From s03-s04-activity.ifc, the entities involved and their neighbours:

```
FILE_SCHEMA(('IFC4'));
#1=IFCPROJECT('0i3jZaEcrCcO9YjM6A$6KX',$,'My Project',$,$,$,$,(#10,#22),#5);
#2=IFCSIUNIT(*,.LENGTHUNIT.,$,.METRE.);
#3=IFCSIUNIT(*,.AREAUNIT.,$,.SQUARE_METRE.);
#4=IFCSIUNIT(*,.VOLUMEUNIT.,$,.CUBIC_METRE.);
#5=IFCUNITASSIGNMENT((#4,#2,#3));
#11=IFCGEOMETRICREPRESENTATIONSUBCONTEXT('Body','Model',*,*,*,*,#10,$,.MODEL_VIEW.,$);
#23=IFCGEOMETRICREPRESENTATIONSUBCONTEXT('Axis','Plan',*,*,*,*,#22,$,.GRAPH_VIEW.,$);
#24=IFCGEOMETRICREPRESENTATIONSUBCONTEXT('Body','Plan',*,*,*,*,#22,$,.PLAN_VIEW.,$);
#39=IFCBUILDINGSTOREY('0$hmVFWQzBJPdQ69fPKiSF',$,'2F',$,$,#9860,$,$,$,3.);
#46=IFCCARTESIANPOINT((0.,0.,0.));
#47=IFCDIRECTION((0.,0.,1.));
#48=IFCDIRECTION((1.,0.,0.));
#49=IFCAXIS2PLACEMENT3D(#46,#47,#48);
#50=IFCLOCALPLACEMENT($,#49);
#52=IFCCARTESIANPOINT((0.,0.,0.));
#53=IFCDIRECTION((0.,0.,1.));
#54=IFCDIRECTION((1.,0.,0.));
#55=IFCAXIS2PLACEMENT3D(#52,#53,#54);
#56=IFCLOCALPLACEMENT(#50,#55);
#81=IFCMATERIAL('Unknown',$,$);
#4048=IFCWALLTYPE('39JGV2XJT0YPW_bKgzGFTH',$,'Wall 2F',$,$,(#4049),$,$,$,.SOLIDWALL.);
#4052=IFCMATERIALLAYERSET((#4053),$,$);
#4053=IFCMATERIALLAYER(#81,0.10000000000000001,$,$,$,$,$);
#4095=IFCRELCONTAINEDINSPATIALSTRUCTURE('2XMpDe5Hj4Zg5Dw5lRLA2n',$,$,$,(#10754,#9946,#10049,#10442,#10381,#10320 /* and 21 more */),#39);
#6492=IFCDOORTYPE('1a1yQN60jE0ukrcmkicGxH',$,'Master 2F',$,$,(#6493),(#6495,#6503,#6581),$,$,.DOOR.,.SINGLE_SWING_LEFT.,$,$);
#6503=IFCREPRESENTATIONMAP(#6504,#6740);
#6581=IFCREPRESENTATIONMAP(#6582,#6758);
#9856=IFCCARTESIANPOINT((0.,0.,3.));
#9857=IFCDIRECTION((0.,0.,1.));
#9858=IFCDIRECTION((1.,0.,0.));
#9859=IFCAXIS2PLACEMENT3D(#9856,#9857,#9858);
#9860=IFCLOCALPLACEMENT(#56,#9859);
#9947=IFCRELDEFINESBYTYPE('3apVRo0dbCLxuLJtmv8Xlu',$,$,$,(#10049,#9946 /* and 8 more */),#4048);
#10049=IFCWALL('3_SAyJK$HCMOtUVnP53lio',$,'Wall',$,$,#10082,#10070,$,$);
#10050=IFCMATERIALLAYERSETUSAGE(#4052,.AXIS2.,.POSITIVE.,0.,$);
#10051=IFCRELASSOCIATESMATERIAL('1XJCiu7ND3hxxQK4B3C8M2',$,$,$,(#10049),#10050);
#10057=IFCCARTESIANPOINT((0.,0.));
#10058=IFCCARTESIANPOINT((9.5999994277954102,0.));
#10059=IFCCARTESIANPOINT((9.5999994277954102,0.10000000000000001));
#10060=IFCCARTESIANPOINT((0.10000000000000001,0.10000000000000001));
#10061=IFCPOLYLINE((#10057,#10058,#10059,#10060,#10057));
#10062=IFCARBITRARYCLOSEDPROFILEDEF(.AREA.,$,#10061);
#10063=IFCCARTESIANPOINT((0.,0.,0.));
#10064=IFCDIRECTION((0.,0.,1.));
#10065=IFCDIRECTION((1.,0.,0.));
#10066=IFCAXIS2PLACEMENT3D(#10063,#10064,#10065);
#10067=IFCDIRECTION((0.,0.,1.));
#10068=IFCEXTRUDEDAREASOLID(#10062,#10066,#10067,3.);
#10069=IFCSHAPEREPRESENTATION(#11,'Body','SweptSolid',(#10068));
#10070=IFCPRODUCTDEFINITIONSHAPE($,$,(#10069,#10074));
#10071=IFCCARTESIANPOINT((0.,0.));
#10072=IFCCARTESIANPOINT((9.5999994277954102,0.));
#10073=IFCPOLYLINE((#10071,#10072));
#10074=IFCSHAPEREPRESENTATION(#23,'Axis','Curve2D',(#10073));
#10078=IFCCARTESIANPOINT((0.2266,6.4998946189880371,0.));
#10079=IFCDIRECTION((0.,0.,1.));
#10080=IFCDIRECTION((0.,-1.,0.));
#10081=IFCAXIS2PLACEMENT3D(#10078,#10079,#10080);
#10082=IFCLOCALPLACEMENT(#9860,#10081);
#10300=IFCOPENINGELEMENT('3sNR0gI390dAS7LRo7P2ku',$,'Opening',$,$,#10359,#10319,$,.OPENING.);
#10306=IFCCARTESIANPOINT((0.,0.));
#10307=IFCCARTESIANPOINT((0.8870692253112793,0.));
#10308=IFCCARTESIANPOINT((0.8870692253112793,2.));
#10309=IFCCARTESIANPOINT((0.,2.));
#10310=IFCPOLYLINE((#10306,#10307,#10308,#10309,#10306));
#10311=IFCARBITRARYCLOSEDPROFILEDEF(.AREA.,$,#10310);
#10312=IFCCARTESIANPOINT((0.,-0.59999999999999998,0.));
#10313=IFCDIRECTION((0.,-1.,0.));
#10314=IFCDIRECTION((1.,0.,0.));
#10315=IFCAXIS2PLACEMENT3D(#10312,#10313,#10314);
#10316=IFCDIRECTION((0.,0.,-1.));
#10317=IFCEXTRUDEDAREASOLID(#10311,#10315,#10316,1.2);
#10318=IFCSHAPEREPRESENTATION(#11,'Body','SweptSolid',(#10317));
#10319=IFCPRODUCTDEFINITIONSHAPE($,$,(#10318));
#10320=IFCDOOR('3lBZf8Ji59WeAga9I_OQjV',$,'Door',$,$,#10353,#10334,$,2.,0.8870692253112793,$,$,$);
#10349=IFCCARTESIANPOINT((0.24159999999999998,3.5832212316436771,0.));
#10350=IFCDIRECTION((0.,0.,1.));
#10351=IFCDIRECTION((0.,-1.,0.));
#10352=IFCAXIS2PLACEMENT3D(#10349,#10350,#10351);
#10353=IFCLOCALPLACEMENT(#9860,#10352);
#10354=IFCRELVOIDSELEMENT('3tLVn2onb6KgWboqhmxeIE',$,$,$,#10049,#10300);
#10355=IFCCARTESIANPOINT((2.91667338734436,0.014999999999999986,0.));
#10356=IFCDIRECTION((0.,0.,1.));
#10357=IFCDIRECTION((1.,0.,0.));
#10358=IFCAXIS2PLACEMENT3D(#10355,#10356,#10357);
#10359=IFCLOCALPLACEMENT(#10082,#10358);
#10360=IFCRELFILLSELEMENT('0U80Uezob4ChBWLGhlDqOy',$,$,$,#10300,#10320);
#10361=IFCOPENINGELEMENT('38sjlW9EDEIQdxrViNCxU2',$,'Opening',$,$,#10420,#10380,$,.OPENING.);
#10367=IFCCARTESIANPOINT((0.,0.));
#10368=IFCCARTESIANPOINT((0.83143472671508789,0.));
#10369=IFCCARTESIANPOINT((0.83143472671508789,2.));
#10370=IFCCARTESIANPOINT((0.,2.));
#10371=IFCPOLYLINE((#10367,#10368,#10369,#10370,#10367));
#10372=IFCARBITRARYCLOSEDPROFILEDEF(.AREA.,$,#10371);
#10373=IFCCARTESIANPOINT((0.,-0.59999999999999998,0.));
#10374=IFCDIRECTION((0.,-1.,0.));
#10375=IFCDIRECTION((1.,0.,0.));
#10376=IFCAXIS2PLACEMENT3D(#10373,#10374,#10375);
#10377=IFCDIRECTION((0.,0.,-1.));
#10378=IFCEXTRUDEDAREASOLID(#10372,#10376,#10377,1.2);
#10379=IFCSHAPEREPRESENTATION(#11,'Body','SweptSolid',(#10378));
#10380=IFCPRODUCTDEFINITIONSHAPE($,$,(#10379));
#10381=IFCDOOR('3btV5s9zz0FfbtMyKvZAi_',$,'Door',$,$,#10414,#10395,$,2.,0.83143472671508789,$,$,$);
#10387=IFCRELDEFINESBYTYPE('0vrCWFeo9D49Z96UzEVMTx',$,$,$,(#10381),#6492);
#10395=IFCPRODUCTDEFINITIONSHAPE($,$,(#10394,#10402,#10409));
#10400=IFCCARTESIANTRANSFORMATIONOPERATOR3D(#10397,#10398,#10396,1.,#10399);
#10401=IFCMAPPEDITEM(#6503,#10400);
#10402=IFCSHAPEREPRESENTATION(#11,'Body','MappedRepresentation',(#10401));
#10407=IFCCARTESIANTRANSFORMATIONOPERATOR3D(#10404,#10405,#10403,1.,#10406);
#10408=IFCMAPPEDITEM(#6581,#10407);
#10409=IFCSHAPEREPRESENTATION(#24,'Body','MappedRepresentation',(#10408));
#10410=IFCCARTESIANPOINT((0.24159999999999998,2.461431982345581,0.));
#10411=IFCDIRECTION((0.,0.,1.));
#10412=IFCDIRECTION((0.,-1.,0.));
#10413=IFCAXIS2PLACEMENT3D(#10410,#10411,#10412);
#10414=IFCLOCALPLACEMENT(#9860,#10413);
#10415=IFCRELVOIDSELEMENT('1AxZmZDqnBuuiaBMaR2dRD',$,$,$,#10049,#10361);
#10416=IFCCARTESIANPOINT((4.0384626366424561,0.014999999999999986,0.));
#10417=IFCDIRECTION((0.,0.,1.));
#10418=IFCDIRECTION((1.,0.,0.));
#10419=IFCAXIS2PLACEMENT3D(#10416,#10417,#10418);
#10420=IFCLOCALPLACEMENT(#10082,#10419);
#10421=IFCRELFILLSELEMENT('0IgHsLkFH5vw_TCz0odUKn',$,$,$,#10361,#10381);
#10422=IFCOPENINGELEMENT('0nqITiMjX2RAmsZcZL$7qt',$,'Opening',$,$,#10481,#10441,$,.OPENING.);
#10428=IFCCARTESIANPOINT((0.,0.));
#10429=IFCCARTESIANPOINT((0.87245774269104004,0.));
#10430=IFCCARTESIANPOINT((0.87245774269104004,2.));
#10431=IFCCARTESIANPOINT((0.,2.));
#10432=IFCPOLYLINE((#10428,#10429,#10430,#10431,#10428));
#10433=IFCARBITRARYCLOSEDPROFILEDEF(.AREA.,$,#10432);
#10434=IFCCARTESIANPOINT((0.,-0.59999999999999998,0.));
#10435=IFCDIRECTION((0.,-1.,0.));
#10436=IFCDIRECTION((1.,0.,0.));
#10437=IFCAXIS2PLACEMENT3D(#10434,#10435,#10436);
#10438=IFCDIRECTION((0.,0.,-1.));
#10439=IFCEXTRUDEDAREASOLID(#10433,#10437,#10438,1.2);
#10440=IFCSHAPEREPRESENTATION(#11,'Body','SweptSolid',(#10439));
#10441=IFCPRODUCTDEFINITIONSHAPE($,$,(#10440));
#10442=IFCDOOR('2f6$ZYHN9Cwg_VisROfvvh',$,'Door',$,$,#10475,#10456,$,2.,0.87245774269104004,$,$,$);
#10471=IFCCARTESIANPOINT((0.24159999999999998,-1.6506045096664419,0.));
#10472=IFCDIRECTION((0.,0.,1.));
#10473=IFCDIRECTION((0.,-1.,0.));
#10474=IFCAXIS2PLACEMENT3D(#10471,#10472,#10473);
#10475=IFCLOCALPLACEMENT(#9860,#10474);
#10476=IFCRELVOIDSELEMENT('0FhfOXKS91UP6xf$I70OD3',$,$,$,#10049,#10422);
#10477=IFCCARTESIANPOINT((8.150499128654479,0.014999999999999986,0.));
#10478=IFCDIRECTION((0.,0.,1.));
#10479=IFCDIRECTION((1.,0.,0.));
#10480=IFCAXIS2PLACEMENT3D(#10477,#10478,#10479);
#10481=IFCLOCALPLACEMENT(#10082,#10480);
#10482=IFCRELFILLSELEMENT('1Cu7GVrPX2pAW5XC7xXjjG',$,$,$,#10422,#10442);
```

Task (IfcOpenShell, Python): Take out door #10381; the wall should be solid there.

```python
import ifcopenshell
import ifcopenshell.api.feature
import ifcopenshell.api.root
import ifcopenshell.geom
import ifcopenshell.util.shape

model = ifcopenshell.open("s03-s04-activity.ifc")
settings = ifcopenshell.geom.settings()


def volume(element):
    """Net volume in cubic metres, openings subtracted."""
    shape = ifcopenshell.geom.create_shape(settings, element)
    return ifcopenshell.util.shape.get_volume(shape.geometry)


door = model.by_guid("3btV5s9zz0FfbtMyKvZAi_")
opening = door.FillsVoids[0].RelatingOpeningElement
wall = opening.VoidsElements[0].RelatingBuildingElement
before = volume(wall)

ifcopenshell.api.root.remove_product(model, product=door)
ifcopenshell.api.feature.remove_feature(model, feature=opening)

after = volume(wall)

print(f"wall volume {before:.3f} -> {after:.3f} m3")

model.write("s03-s04-activity_v2.ifc")
```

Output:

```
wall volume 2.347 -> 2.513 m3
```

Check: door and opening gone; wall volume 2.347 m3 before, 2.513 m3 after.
